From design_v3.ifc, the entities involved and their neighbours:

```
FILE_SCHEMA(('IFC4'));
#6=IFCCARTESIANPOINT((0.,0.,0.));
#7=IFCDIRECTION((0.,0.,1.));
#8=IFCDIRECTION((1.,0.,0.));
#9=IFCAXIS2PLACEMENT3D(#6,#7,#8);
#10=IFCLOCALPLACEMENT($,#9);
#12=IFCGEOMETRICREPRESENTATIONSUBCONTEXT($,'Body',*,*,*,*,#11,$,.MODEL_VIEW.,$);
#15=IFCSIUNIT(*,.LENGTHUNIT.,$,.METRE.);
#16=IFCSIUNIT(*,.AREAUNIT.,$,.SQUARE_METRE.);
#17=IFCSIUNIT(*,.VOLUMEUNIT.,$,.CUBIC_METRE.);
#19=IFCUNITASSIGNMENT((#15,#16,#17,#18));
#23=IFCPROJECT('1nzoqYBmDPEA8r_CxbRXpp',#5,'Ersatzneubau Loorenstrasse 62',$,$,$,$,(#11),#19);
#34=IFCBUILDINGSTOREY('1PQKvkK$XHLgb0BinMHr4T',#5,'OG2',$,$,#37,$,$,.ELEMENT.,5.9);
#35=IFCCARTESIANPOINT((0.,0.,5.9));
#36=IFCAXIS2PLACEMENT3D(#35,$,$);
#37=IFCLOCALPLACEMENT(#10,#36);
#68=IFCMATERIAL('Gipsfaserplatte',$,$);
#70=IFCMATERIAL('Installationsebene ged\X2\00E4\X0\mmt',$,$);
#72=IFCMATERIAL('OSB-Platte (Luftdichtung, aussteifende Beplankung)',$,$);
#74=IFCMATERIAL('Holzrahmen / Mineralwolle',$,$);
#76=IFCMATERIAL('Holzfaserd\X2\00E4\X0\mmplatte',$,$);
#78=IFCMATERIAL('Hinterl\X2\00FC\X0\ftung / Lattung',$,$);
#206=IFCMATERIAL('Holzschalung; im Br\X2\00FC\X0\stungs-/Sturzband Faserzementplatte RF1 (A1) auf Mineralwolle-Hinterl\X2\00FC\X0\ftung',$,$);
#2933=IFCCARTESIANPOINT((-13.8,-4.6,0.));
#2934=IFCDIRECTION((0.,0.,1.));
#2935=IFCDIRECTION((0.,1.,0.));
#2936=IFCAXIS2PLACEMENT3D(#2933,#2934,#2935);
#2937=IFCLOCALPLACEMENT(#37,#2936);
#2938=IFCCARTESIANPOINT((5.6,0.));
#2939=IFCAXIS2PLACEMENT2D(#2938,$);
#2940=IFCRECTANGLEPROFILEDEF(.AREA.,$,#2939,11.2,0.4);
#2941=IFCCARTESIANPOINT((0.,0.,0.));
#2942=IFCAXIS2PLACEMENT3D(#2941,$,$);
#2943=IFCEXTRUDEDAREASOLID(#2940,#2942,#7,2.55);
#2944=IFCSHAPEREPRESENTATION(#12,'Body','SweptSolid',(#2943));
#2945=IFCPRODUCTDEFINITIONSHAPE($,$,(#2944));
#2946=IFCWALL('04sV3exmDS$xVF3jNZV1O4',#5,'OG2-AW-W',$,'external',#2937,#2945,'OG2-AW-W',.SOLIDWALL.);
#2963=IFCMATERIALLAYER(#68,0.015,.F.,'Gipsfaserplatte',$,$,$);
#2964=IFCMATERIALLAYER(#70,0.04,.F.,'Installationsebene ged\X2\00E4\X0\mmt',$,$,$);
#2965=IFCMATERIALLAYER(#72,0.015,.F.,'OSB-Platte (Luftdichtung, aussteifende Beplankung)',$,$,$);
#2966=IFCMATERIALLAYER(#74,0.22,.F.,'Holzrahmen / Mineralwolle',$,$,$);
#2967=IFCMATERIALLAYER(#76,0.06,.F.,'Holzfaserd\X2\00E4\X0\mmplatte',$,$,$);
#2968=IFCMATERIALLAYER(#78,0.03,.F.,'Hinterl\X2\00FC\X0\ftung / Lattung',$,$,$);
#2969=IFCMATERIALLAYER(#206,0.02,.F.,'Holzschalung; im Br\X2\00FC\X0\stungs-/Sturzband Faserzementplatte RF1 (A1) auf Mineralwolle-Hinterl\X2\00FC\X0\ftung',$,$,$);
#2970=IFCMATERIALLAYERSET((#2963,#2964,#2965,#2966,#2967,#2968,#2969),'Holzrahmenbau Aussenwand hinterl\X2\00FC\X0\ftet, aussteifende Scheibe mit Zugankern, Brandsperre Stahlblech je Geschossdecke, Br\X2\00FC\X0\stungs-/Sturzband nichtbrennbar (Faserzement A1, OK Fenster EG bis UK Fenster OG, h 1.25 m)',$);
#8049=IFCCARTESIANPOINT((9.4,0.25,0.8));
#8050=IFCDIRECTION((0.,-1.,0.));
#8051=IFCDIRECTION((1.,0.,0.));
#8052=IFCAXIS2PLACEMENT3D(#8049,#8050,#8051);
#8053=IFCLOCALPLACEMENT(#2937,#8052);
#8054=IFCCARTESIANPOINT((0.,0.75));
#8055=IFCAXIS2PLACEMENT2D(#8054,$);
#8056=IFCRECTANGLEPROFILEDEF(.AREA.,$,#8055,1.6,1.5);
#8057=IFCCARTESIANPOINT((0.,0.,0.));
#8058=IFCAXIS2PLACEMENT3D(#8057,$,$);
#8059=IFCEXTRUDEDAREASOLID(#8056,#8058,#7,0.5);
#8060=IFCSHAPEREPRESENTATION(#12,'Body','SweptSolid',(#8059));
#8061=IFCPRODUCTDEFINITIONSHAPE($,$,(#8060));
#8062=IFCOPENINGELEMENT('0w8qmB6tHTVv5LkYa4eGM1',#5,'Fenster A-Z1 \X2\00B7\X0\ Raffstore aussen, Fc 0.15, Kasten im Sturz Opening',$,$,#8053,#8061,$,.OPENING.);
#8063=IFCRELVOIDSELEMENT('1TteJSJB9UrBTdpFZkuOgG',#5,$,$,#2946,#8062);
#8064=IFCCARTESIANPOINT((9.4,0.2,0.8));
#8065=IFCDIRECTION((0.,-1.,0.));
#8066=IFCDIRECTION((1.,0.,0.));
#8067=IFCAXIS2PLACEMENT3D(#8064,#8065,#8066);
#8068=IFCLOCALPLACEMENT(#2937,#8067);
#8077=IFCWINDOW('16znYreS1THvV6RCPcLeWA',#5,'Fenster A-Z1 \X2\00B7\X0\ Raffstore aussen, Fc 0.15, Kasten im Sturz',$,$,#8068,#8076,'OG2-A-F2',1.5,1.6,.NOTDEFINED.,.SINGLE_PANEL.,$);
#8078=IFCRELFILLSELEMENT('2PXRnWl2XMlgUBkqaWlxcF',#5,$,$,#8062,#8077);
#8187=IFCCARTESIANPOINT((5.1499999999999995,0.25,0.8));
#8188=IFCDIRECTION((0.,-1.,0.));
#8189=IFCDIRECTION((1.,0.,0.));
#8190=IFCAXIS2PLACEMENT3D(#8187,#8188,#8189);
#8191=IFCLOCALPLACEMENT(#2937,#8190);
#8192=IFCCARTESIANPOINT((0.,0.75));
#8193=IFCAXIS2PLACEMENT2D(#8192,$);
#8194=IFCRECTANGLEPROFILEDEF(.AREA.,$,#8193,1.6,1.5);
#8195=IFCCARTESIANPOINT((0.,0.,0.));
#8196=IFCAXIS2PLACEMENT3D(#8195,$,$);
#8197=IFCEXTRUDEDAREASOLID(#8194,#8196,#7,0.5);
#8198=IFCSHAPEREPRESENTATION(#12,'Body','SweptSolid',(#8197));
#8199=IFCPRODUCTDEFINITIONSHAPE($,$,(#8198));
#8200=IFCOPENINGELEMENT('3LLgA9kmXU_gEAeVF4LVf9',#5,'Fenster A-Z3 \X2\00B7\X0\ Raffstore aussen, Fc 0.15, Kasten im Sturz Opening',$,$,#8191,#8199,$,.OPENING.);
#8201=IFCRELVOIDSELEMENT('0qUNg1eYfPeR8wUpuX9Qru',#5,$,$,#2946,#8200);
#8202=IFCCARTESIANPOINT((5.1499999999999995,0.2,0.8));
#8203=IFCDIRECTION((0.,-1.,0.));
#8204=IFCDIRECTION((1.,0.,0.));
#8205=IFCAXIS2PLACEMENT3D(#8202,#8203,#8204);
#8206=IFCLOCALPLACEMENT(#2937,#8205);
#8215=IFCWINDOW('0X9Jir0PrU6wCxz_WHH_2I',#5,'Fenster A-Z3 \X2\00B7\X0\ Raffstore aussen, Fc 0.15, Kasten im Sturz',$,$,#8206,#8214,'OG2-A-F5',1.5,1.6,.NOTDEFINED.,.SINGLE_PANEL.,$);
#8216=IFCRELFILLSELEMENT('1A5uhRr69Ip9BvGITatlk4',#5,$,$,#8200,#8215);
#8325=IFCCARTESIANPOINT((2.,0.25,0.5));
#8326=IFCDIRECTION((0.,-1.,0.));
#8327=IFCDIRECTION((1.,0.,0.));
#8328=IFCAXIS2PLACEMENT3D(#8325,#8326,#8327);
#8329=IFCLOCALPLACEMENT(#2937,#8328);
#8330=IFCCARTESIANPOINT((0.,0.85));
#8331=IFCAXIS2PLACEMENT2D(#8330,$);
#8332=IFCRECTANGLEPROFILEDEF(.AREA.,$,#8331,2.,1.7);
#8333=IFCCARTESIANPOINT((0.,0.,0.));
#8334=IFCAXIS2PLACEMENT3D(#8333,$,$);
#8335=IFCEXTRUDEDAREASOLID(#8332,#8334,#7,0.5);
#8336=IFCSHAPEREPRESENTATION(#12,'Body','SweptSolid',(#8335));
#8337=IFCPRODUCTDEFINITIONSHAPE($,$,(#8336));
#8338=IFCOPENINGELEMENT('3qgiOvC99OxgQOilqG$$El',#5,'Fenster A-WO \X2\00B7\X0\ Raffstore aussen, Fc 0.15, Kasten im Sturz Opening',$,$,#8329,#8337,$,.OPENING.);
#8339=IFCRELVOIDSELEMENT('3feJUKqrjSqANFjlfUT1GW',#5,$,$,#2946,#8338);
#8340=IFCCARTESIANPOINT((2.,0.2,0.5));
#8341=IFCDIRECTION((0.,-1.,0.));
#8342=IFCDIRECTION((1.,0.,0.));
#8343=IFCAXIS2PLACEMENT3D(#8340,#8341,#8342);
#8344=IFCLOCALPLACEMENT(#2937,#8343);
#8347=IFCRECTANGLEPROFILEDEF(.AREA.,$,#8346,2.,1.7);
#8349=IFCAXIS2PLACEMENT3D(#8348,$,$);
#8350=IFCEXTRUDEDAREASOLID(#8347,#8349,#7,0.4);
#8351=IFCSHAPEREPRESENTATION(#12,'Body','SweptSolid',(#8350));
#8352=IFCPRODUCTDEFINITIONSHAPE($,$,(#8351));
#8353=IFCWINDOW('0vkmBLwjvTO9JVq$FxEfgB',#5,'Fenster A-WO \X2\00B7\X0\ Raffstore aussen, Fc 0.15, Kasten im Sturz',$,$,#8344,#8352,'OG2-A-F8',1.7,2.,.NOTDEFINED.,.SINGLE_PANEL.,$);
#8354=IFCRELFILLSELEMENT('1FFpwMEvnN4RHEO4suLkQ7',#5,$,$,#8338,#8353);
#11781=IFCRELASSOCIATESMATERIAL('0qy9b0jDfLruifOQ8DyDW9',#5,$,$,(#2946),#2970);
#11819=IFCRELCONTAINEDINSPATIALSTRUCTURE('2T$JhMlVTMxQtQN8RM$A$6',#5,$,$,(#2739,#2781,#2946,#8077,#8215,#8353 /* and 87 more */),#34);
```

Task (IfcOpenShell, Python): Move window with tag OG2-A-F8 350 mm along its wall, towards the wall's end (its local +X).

```python
import ifcopenshell
import ifcopenshell.api.geometry
import ifcopenshell.util.placement

model = ifcopenshell.open("design_v3.ifc")

window = model.by_guid("0vkmBLwjvTO9JVq$FxEfgB")
opening = window.FillsVoids[0].RelatingOpeningElement
wall = opening.VoidsElements[0].RelatingBuildingElement

wall_matrix = ifcopenshell.util.placement.get_local_placement(wall.ObjectPlacement)
shift = wall_matrix[:3, 0] * 0.35
before = ifcopenshell.util.placement.get_local_placement(window.ObjectPlacement)[:3, 3].copy()

# The window is not placed relative to its opening, so move both.
for product in (opening, window):
    matrix = ifcopenshell.util.placement.get_local_placement(product.ObjectPlacement)
    matrix[:3, 3] += shift
    ifcopenshell.api.geometry.edit_object_placement(model, product=product, matrix=matrix, is_si=False)

after = ifcopenshell.util.placement.get_local_placement(window.ObjectPlacement)[:3, 3]
print("window moved by", (after - before).round(3) + 0.0)

model.write("design_v3_v2.ifc")
```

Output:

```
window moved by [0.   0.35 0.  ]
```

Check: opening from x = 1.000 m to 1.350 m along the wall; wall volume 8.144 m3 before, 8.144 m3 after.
